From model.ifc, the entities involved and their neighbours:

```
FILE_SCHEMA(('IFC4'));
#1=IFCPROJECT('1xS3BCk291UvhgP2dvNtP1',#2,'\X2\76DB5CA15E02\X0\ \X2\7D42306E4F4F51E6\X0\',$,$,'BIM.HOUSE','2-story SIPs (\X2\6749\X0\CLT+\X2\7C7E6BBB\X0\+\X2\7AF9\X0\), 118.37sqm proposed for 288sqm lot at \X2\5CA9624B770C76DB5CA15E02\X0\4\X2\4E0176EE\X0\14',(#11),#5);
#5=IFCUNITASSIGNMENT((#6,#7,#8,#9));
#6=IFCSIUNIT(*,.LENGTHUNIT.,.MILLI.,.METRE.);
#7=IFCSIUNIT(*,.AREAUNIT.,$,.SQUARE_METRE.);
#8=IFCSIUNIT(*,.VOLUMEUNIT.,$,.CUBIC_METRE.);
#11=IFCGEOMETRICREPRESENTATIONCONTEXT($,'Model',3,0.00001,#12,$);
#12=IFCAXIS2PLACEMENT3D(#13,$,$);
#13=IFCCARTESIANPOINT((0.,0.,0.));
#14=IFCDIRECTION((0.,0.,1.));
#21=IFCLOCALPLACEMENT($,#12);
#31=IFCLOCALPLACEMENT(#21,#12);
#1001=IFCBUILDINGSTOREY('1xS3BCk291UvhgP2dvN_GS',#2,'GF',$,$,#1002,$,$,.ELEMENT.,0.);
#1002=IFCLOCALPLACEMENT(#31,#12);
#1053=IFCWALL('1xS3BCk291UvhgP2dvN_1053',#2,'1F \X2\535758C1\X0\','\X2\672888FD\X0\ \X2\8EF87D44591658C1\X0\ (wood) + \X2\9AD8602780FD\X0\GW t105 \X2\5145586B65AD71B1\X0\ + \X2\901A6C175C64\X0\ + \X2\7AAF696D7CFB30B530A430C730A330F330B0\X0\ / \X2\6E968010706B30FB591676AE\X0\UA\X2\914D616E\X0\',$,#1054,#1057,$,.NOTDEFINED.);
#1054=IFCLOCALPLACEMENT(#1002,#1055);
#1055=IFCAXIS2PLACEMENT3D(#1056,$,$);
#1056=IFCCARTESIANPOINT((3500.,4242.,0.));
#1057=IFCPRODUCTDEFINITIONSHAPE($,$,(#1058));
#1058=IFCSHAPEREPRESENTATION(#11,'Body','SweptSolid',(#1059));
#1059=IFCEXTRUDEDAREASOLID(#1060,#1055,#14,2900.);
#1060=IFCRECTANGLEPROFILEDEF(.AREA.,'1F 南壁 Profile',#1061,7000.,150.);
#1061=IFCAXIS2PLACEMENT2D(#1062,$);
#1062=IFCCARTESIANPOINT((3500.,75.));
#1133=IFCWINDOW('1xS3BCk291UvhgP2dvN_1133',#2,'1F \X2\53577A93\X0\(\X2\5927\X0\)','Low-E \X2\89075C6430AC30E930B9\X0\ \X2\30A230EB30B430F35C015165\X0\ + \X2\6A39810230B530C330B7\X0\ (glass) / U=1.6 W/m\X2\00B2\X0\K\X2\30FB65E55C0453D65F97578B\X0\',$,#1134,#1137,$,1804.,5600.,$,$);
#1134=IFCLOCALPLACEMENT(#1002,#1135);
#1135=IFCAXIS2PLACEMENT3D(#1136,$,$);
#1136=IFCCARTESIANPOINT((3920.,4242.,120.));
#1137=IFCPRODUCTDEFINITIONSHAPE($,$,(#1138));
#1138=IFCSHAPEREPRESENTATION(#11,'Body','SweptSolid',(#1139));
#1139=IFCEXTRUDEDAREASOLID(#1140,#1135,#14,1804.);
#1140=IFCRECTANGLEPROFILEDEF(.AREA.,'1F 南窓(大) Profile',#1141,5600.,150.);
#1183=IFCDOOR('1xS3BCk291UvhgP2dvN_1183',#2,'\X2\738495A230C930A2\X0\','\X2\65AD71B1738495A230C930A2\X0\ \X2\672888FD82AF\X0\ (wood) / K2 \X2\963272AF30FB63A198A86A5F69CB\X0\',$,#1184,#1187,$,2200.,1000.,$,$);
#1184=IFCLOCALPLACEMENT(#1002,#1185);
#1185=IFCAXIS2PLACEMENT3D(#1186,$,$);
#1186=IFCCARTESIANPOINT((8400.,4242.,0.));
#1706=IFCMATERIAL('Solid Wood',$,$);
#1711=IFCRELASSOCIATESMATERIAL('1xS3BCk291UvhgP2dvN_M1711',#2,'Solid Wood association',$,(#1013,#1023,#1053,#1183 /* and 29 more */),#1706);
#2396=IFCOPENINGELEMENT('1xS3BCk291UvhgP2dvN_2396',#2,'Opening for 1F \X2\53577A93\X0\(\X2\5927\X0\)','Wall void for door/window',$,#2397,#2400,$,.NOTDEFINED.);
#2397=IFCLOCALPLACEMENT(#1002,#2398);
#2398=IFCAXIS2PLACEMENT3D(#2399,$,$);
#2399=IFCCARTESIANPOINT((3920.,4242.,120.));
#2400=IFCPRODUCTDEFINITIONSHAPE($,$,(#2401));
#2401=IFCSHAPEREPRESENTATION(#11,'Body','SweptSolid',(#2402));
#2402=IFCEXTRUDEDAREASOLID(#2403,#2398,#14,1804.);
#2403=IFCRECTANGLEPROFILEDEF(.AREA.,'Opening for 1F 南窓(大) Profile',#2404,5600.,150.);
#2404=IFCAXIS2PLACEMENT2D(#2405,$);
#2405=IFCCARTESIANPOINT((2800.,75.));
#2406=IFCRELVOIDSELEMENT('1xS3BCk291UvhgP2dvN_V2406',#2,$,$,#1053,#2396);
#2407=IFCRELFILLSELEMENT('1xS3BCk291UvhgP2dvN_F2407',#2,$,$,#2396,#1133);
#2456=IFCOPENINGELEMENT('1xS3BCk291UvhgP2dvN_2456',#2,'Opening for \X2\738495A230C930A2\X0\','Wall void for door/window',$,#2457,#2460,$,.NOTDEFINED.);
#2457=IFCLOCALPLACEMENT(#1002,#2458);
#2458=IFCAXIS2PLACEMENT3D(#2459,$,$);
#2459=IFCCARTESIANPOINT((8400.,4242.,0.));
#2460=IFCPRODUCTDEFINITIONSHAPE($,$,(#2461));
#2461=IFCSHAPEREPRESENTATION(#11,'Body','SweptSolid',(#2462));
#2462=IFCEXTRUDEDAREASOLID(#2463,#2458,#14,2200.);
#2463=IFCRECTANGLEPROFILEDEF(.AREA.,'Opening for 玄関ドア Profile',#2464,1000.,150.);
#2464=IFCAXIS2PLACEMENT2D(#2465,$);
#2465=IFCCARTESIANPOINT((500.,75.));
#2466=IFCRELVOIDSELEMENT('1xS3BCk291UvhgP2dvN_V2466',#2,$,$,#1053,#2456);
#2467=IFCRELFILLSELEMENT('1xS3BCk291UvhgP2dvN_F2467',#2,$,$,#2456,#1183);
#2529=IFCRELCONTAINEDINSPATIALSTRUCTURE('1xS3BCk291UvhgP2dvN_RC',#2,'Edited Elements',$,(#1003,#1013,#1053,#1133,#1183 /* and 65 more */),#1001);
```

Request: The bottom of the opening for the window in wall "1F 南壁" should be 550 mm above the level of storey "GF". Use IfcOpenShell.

```python
import numpy as np
import ifcopenshell
import ifcopenshell.api.geometry
import ifcopenshell.geom
import ifcopenshell.util.element
import ifcopenshell.util.placement
import ifcopenshell.util.shape
import ifcopenshell.util.unit

model = ifcopenshell.open("model.ifc")
unit_scale = ifcopenshell.util.unit.calculate_unit_scale(model)

window = model.by_guid("1xS3BCk291UvhgP2dvN_1133")
opening = window.FillsVoids[0].RelatingOpeningElement
storey = ifcopenshell.util.element.get_container(window, ifc_class="IfcBuildingStorey")
level = ifcopenshell.util.placement.get_local_placement(storey.ObjectPlacement)[2, 3]

# The opening's origin need not be at the sill, so measure its lowest point.
shape = ifcopenshell.geom.create_shape(ifcopenshell.geom.settings(), opening)
bottom = ifcopenshell.util.shape.get_shape_bottom_elevation(shape, shape.geometry) / unit_scale
dz = level + 0.55 / unit_scale - bottom

shift = np.array([0.0, 0.0, dz])
# The window is not placed relative to its opening, so move both.
for product in (opening, window):
    matrix = ifcopenshell.util.placement.get_local_placement(product.ObjectPlacement)
    matrix[:3, 3] += shift
    ifcopenshell.api.geometry.edit_object_placement(model, product=product, matrix=matrix, is_si=False)

print(f"moved by {dz * unit_scale:+.3f} m")

model.write("model_edited.ifc")
```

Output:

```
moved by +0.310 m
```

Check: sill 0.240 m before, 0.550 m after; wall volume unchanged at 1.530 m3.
